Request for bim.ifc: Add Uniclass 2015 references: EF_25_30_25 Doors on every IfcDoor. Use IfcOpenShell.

First a look at what the model holds.

```python
import ifcopenshell

model = ifcopenshell.open("bim.ifc")
print(model.schema)
print("classifications:", [c.Name for c in model.by_type("IfcClassification")])
for ifc_class in ("IfcDoor", "IfcRoof", "IfcStair", "IfcWall", "IfcWindow"):
    print(ifc_class, len(model.by_type(ifc_class)))
```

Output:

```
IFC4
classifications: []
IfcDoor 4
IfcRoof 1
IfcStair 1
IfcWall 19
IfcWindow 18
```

```python
import ifcopenshell
import ifcopenshell.api.classification

model = ifcopenshell.open("bim.ifc")

system = ifcopenshell.api.classification.add_classification(model, classification="Uniclass 2015")

codes = {
    "IfcDoor": ("EF_25_30_25", "Doors"),
}
for ifc_class, (code, name) in codes.items():
    products = model.by_type(ifc_class)
    ifcopenshell.api.classification.add_reference(
        model, products=products, classification=system, identification=code, name=name
    )
    print(code, len(products))

model.write("bim_v2.ifc")
```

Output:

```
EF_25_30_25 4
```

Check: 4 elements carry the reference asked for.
